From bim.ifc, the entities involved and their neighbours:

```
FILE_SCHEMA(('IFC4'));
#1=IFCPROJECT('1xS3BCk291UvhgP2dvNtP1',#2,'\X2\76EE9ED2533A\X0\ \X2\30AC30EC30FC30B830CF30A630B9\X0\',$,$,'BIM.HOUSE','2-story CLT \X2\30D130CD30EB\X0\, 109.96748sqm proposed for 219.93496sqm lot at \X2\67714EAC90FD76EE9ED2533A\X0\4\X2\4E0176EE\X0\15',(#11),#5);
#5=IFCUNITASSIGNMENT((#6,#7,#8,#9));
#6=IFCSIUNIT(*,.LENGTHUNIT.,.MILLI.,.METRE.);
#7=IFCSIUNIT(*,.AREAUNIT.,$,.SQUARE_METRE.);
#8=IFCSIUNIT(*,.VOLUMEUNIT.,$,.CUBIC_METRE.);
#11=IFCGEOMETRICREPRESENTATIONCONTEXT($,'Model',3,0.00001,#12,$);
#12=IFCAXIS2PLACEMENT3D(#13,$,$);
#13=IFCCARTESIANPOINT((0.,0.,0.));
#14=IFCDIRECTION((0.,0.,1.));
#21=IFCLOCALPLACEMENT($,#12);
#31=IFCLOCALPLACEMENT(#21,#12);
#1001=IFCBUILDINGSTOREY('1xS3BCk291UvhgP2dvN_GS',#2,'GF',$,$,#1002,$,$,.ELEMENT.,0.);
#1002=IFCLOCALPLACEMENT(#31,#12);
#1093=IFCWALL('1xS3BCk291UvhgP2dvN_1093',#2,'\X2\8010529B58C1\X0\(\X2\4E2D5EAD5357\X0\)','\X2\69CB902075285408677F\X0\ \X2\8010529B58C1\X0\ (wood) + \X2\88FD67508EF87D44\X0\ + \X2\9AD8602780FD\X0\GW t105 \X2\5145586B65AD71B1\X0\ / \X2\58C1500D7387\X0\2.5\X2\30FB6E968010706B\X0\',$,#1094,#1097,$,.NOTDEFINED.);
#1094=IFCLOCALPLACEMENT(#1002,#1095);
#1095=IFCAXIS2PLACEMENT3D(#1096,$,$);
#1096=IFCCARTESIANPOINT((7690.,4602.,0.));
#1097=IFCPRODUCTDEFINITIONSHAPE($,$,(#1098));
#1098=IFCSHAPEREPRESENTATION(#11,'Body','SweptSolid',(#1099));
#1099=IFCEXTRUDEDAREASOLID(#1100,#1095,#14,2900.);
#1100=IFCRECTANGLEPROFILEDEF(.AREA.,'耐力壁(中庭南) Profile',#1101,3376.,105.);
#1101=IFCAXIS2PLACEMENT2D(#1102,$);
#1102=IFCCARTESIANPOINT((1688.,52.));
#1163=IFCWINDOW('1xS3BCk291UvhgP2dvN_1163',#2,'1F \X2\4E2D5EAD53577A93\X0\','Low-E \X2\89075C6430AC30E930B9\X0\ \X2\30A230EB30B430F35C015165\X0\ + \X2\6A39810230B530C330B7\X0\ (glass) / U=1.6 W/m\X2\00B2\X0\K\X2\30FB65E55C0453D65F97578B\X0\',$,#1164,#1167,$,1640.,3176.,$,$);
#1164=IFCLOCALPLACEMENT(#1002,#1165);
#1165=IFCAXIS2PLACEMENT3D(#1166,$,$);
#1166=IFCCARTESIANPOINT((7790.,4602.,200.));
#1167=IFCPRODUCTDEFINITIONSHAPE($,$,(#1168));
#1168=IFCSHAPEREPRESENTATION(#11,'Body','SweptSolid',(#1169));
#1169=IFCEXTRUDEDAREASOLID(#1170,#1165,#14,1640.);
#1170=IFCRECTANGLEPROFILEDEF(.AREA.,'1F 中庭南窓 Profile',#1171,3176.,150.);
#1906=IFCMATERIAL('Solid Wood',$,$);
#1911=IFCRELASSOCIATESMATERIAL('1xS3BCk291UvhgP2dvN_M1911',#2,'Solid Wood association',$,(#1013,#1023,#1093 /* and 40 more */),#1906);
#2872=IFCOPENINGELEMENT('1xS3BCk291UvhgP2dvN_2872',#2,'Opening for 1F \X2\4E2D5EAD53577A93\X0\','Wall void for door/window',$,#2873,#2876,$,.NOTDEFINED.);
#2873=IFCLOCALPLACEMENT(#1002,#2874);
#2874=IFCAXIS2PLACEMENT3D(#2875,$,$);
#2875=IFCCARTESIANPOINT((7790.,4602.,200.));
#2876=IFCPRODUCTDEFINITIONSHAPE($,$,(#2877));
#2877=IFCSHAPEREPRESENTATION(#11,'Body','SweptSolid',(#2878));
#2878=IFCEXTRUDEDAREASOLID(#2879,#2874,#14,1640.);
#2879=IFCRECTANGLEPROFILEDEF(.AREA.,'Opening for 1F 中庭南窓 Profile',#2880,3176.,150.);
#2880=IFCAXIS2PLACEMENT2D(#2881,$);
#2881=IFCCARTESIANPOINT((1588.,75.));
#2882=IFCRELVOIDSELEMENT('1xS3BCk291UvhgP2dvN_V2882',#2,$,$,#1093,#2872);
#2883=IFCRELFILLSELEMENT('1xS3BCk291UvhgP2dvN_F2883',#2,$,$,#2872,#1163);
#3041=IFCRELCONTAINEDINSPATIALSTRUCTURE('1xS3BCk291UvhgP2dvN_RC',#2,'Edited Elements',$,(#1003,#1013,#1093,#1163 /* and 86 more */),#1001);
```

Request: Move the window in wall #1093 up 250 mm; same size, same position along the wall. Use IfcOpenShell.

```python
import numpy as np
import ifcopenshell
import ifcopenshell.api.geometry
import ifcopenshell.util.placement
import ifcopenshell.util.unit

model = ifcopenshell.open("bim.ifc")
unit_scale = ifcopenshell.util.unit.calculate_unit_scale(model)

window = model.by_guid("1xS3BCk291UvhgP2dvN_1163")
opening = window.FillsVoids[0].RelatingOpeningElement
dz = 0.25 / unit_scale

shift = np.array([0.0, 0.0, dz])
# The window is not placed relative to its opening, so move both.
for product in (opening, window):
    matrix = ifcopenshell.util.placement.get_local_placement(product.ObjectPlacement)
    matrix[:3, 3] += shift
    ifcopenshell.api.geometry.edit_object_placement(model, product=product, matrix=matrix, is_si=False)

print(f"moved by {dz * unit_scale:+.3f} m")

model.write("bim_updated.ifc")
```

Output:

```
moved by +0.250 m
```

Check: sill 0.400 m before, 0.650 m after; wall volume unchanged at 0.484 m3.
